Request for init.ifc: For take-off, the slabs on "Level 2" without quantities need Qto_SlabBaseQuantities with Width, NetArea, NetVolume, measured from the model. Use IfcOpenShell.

First a look at what the model holds.

```python
import ifcopenshell
import ifcopenshell.util.element
import ifcopenshell.util.unit

model = ifcopenshell.open("init.ifc")
print(model.schema)
for unit_type in ("LENGTHUNIT", "AREAUNIT", "VOLUMEUNIT"):
    print(unit_type, ifcopenshell.util.unit.calculate_unit_scale(model, unit_type))
storey = next(s for s in model.by_type("IfcBuildingStorey") if s.Name == "Level 2")
slabs = [e for e in ifcopenshell.util.element.get_decomposition(storey) if e.is_a("IfcSlab")]
for e in sorted(slabs, key=lambda e: e.id()):
    print(e.id(), e.is_a(), e.Name, list(ifcopenshell.util.element.get_psets(e, qtos_only=True)), sep=" | ")
```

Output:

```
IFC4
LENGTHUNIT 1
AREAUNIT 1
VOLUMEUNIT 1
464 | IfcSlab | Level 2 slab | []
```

```python
import ifcopenshell
import ifcopenshell.api.pset
import ifcopenshell.geom
import ifcopenshell.util.element
import ifcopenshell.util.shape
import ifcopenshell.util.unit

model = ifcopenshell.open("init.ifc")
unit_scale = ifcopenshell.util.unit.calculate_unit_scale(model)
area_scale = ifcopenshell.util.unit.calculate_unit_scale(model, "AREAUNIT")
volume_scale = ifcopenshell.util.unit.calculate_unit_scale(model, "VOLUMEUNIT")
settings = ifcopenshell.geom.settings()

storey = next(s for s in model.by_type("IfcBuildingStorey") if s.Name == "Level 2")
slabs = [e for e in ifcopenshell.util.element.get_decomposition(storey) if e.is_a("IfcSlab")]

for e in sorted(slabs, key=lambda e: e.id()):
    if ifcopenshell.util.element.get_psets(e, qtos_only=True, should_inherit=False):
        continue
    # Geometry comes back in metres, in the element's own axes.
    shape = ifcopenshell.geom.create_shape(settings, e)
    values = {
        "Width": ifcopenshell.util.shape.get_z(shape.geometry) / unit_scale,
        "NetArea": ifcopenshell.util.shape.get_footprint_area(shape.geometry) / area_scale,
        "NetVolume": ifcopenshell.util.shape.get_volume(shape.geometry) / volume_scale,
    }
    qto = ifcopenshell.api.pset.add_qto(model, product=e, name="Qto_SlabBaseQuantities")
    ifcopenshell.api.pset.edit_qto(model, qto=qto, properties=values)
    print(e.id(), {k: round(v, 3) for k, v in values.items()})

model.write("init_v2.ifc")
```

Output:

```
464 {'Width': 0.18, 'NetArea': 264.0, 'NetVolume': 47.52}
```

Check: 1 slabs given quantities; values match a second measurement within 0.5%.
